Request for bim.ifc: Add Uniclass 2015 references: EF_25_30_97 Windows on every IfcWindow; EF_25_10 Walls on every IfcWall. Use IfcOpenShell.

First a look at what the model holds.

```python
import ifcopenshell

model = ifcopenshell.open("bim.ifc")
print(model.schema)
print("classifications:", [c.Name for c in model.by_type("IfcClassification")])
for ifc_class in ("IfcDoor", "IfcRoof", "IfcStair", "IfcWall", "IfcWindow"):
    print(ifc_class, len(model.by_type(ifc_class)))
```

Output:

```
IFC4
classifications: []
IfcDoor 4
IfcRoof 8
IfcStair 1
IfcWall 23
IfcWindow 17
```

```python
import ifcopenshell
import ifcopenshell.api.classification

model = ifcopenshell.open("bim.ifc")

system = ifcopenshell.api.classification.add_classification(model, classification="Uniclass 2015")

codes = {
    "IfcWindow": ("EF_25_30_97", "Windows"),
    "IfcWall": ("EF_25_10", "Walls"),
}
for ifc_class, (code, name) in codes.items():
    products = model.by_type(ifc_class)
    ifcopenshell.api.classification.add_reference(
        model, products=products, classification=system, identification=code, name=name
    )
    print(code, len(products))

model.write("bim_v2.ifc")
```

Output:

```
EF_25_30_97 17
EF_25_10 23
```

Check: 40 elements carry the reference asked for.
